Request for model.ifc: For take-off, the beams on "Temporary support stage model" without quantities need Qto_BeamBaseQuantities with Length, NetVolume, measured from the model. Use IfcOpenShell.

First a look at what the model holds.

```python
import ifcopenshell
import ifcopenshell.util.element
import ifcopenshell.util.unit

model = ifcopenshell.open("model.ifc")
print(model.schema)
for unit_type in ("LENGTHUNIT", "AREAUNIT", "VOLUMEUNIT"):
    print(unit_type, ifcopenshell.util.unit.calculate_unit_scale(model, unit_type))
storey = next(s for s in model.by_type("IfcBuildingStorey") if s.Name == "Temporary support stage model")
beams = [e for e in ifcopenshell.util.element.get_decomposition(storey) if e.is_a("IfcBeam")]
for e in sorted(beams, key=lambda e: e.id()):
    print(e.id(), e.is_a(), e.Name, list(ifcopenshell.util.element.get_psets(e, qtos_only=True)), sep=" | ")
```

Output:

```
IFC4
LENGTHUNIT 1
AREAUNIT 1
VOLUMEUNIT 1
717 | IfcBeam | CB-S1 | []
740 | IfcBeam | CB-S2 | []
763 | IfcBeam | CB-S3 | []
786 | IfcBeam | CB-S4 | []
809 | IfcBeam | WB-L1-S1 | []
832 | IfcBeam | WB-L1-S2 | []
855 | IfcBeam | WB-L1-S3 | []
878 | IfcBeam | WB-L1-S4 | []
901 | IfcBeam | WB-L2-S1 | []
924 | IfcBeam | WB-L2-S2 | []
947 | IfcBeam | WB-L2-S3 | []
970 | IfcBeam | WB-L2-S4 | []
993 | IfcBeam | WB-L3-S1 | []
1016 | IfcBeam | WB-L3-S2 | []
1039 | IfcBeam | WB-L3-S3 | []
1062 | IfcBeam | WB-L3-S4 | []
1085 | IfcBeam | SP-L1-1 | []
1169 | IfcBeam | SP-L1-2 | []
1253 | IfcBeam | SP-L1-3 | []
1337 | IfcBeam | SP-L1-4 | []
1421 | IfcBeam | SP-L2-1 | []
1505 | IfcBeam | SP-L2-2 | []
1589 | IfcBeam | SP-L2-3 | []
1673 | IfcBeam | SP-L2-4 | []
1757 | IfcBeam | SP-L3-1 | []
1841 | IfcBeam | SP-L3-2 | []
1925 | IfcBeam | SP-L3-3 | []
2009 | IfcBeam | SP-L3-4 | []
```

```python
import ifcopenshell
import ifcopenshell.api.pset
import ifcopenshell.geom
import ifcopenshell.util.element
import ifcopenshell.util.shape
import ifcopenshell.util.unit

model = ifcopenshell.open("model.ifc")
unit_scale = ifcopenshell.util.unit.calculate_unit_scale(model)
volume_scale = ifcopenshell.util.unit.calculate_unit_scale(model, "VOLUMEUNIT")
settings = ifcopenshell.geom.settings()

storey = next(s for s in model.by_type("IfcBuildingStorey") if s.Name == "Temporary support stage model")
beams = [e for e in ifcopenshell.util.element.get_decomposition(storey) if e.is_a("IfcBeam")]

for e in sorted(beams, key=lambda e: e.id()):
    if ifcopenshell.util.element.get_psets(e, qtos_only=True, should_inherit=False):
        continue
    # Geometry comes back in metres, in the element's own axes.
    shape = ifcopenshell.geom.create_shape(settings, e)
    values = {
        "Length": ifcopenshell.util.shape.get_max_xyz(shape.geometry) / unit_scale,
        "NetVolume": ifcopenshell.util.shape.get_volume(shape.geometry) / volume_scale,
    }
    qto = ifcopenshell.api.pset.add_qto(model, product=e, name="Qto_BeamBaseQuantities")
    ifcopenshell.api.pset.edit_qto(model, qto=qto, properties=values)
    print(e.id(), {k: round(v, 3) for k, v in values.items()})

model.write("model_rev.ifc")
```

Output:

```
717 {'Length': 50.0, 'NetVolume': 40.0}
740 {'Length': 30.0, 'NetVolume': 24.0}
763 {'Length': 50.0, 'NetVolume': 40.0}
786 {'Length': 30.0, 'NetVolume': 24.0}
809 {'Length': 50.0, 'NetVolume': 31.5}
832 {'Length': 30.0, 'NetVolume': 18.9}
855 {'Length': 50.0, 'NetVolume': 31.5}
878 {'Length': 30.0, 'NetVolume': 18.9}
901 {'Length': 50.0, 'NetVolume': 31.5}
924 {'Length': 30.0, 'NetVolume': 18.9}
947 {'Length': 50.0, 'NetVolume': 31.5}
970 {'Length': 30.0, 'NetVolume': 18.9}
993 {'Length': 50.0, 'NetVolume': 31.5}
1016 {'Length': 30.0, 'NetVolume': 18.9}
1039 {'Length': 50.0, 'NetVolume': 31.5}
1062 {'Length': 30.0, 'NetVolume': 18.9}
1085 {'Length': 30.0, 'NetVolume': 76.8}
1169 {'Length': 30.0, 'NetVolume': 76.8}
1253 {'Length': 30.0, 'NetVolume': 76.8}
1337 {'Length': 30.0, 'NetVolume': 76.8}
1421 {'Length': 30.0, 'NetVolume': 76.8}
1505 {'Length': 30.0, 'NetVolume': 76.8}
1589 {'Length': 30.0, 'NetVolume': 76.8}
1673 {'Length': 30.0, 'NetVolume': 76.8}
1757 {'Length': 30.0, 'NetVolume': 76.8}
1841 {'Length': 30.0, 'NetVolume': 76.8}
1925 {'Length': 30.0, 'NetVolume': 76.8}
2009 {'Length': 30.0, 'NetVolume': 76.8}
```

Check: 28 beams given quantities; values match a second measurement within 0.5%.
